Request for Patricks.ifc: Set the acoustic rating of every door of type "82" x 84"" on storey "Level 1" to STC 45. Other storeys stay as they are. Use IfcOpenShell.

First a look at what the model holds.

```python
import ifcopenshell
import ifcopenshell.util.element

model = ifcopenshell.open("Patricks.ifc")
print(model.schema)
storey = next(s for s in model.by_type("IfcBuildingStorey") if s.Name == "Level 1")
doors = [e for e in ifcopenshell.util.element.get_decomposition(storey) if e.is_a("IfcDoor")]
seen = {}
for e in doors:
    element_type = ifcopenshell.util.element.get_type(e)
    key = (element_type.Name if element_type != e and element_type else None, ifcopenshell.util.element.get_pset(e, "Pset_DoorCommon", "AcousticRating"))
    seen[key] = seen.get(key, 0) + 1
for (name, value), count in sorted(seen.items(), key=str):
    print(count, "x", name, "|", value)
```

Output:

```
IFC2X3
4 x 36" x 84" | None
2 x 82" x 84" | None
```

```python
import ifcopenshell
import ifcopenshell.api.pset
import ifcopenshell.util.element

model = ifcopenshell.open("Patricks.ifc")

storey = next(s for s in model.by_type("IfcBuildingStorey") if s.Name == "Level 1")
doors = [e for e in ifcopenshell.util.element.get_decomposition(storey) if e.is_a("IfcDoor")]

count = 0
for e in doors:
    element_type = ifcopenshell.util.element.get_type(e)
    if element_type in (None, e) or element_type.Name != '82" x 84"':
        continue
    # add_pset returns the element's existing set when there is one.
    pset = ifcopenshell.api.pset.add_pset(model, product=e, name="Pset_DoorCommon")
    ifcopenshell.api.pset.edit_pset(model, pset=pset, properties={"AcousticRating": "STC 45"})
    count += 1

print(count, "doors updated")

model.write("Patricks_v2.ifc")
```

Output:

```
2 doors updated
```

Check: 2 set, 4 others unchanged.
